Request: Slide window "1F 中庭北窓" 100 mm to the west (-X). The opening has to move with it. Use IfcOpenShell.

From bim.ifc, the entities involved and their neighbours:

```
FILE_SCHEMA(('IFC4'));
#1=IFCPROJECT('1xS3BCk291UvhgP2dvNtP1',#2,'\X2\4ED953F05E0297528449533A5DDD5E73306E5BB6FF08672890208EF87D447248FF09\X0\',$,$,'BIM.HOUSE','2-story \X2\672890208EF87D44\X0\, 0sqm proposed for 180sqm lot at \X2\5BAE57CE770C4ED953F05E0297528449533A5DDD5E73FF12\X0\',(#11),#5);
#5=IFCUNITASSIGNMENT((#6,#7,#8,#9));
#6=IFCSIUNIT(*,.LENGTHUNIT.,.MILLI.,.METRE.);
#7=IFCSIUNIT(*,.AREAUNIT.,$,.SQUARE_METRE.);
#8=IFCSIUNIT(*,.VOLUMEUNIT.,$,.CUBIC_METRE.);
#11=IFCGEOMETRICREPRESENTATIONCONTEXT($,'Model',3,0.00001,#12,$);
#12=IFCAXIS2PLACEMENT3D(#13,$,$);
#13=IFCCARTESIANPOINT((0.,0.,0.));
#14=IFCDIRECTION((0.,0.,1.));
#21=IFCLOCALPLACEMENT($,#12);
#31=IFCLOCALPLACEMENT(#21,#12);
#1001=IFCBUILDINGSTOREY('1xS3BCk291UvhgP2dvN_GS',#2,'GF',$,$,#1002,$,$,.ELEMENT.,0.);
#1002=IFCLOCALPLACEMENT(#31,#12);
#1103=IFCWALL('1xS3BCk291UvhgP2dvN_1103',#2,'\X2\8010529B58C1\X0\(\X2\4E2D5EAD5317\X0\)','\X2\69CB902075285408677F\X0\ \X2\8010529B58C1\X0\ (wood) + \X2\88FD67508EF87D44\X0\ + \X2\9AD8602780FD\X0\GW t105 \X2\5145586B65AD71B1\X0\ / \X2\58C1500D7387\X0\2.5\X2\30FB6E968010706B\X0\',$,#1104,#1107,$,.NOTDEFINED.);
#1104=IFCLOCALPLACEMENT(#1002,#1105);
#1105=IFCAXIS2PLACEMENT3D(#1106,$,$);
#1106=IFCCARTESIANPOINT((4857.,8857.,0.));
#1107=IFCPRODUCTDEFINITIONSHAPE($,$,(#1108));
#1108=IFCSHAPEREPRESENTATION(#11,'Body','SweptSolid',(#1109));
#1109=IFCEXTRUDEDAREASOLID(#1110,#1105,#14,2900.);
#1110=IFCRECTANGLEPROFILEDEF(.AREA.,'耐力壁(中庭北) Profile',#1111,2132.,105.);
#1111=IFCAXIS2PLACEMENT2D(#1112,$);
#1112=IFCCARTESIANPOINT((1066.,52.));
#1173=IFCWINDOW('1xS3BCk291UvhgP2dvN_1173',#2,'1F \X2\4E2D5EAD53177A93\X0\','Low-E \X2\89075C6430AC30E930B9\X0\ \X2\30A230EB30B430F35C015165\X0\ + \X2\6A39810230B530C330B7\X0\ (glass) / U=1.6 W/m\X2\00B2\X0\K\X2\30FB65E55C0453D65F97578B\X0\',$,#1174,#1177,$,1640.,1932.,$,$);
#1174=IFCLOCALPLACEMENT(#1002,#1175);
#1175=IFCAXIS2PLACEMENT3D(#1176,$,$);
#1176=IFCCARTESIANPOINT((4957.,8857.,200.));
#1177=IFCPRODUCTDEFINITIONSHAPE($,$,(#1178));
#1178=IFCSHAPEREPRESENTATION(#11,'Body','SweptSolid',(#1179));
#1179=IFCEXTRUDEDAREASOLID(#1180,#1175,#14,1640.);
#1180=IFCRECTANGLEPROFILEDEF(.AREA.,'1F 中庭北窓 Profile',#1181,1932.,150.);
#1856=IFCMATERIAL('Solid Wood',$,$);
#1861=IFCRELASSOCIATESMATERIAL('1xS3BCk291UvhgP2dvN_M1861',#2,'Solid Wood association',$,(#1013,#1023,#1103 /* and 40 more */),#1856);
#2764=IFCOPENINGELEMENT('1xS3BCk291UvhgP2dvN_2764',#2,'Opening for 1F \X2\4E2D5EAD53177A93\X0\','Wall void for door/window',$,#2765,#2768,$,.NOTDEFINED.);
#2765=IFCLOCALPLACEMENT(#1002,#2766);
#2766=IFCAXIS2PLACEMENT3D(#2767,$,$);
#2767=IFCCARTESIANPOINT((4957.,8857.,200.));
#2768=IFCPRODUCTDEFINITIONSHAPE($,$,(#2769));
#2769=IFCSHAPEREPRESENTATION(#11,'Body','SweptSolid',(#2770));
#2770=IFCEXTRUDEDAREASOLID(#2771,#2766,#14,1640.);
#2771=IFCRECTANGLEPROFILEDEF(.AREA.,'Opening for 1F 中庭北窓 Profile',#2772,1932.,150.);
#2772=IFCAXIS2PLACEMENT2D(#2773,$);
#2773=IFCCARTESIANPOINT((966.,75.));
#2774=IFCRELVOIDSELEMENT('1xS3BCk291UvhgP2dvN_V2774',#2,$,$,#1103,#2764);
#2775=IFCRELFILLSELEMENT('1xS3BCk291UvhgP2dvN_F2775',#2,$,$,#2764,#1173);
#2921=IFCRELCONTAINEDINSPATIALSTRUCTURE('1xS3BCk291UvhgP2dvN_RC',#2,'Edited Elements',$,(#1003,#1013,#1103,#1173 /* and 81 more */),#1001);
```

```python
import ifcopenshell
import ifcopenshell.api.geometry
import ifcopenshell.util.placement
import ifcopenshell.util.unit

model = ifcopenshell.open("bim.ifc")
unit_scale = ifcopenshell.util.unit.calculate_unit_scale(model)

window = model.by_guid("1xS3BCk291UvhgP2dvN_1173")
opening = window.FillsVoids[0].RelatingOpeningElement
wall = opening.VoidsElements[0].RelatingBuildingElement

wall_matrix = ifcopenshell.util.placement.get_local_placement(wall.ObjectPlacement)
shift = wall_matrix[:3, 0] * -0.1 / unit_scale
before = ifcopenshell.util.placement.get_local_placement(window.ObjectPlacement)[:3, 3].copy()

# The window is not placed relative to its opening, so move both.
for product in (opening, window):
    matrix = ifcopenshell.util.placement.get_local_placement(product.ObjectPlacement)
    matrix[:3, 3] += shift
    ifcopenshell.api.geometry.edit_object_placement(model, product=product, matrix=matrix, is_si=False)

after = ifcopenshell.util.placement.get_local_placement(window.ObjectPlacement)[:3, 3]
print("window moved by", (after - before).round(3) + 0.0)

model.write("bim_v2.ifc")
```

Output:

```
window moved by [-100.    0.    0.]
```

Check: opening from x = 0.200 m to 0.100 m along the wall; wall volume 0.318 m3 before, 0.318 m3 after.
